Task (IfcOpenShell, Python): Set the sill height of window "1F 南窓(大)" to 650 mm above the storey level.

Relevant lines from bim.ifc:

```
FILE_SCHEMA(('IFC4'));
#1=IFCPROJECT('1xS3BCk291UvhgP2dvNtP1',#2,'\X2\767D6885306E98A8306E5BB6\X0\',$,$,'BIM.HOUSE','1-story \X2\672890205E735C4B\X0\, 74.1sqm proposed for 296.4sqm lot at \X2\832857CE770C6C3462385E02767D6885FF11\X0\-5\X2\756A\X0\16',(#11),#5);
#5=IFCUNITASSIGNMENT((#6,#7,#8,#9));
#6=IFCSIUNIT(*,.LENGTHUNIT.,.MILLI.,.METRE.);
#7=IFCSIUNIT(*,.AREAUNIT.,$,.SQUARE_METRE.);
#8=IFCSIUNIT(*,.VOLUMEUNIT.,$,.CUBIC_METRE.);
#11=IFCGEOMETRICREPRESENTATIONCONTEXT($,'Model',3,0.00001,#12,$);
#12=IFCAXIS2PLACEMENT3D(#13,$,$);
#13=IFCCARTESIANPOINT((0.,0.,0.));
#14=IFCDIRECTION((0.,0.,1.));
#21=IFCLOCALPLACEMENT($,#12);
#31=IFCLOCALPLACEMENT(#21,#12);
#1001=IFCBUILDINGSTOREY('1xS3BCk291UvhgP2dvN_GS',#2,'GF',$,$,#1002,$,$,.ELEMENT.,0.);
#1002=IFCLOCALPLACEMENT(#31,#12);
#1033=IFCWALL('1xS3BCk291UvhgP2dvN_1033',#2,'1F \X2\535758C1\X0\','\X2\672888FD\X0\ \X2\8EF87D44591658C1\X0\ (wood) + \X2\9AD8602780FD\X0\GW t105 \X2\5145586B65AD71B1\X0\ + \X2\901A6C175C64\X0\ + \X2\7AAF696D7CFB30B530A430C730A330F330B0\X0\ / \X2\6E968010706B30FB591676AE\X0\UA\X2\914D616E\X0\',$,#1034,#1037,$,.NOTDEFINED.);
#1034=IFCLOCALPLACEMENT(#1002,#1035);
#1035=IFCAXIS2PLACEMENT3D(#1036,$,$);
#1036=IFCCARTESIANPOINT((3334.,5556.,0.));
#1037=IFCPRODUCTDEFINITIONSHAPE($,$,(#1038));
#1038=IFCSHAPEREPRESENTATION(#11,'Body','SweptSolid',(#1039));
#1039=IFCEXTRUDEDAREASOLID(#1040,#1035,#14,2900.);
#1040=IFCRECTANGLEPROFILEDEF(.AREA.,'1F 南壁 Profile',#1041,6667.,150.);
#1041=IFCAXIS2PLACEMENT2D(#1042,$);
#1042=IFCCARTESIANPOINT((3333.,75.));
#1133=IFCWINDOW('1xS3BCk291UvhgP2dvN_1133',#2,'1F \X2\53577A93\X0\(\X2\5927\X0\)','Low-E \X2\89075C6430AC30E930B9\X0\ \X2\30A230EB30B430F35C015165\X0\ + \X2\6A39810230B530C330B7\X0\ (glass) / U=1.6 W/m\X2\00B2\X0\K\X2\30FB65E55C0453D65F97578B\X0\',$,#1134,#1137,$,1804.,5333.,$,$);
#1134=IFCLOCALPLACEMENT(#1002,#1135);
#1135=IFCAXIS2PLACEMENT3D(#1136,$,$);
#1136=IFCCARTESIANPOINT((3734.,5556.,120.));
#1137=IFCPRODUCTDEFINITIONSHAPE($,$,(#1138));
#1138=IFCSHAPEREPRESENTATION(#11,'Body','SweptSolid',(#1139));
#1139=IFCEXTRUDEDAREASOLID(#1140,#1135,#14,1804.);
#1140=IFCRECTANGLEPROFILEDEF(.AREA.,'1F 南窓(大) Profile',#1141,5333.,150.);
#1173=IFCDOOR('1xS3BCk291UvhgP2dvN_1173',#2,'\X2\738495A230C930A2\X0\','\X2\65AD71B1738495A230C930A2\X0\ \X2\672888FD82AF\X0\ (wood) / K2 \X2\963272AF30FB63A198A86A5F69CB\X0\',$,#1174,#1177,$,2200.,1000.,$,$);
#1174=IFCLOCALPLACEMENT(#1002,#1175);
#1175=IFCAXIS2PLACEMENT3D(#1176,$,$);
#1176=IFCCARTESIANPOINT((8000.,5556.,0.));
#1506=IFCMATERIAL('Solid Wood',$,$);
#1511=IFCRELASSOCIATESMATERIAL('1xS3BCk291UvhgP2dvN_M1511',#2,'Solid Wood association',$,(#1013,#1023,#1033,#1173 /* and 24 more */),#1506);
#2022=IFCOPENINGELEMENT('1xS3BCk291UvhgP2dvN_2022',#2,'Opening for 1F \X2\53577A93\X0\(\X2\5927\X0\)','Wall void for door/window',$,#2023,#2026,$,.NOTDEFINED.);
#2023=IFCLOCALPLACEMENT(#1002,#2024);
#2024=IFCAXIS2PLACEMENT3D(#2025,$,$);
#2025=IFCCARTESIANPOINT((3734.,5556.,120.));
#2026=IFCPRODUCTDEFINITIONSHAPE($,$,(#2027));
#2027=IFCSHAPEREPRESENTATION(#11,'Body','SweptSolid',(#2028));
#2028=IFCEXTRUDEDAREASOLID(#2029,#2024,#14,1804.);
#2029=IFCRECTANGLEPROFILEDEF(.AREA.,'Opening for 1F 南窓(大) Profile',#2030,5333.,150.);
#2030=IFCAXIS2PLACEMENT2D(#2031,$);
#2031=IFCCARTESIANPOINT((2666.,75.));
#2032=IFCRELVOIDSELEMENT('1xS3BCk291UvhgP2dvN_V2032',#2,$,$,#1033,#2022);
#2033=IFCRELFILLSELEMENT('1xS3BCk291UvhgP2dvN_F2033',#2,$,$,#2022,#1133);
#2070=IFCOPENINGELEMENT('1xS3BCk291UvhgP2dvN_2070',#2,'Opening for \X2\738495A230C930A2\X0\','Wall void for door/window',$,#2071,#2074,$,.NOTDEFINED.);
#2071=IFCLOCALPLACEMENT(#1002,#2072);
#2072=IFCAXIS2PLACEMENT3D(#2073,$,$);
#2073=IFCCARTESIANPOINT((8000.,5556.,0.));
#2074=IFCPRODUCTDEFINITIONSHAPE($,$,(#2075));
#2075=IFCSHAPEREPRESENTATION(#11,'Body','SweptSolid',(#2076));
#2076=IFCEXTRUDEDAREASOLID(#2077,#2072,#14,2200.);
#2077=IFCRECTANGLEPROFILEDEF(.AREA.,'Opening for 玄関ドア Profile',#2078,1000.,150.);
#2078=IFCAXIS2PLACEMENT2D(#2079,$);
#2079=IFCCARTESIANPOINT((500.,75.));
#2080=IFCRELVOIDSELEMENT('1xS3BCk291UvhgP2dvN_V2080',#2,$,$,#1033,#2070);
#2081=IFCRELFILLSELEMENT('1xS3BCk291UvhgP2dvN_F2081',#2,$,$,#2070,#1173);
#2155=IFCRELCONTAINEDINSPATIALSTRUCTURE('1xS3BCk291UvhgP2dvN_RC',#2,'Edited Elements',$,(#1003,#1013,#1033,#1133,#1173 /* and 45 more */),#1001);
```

```python
import numpy as np
import ifcopenshell
import ifcopenshell.api.geometry
import ifcopenshell.geom
import ifcopenshell.util.element
import ifcopenshell.util.placement
import ifcopenshell.util.shape
import ifcopenshell.util.unit

model = ifcopenshell.open("bim.ifc")
unit_scale = ifcopenshell.util.unit.calculate_unit_scale(model)

window = model.by_guid("1xS3BCk291UvhgP2dvN_1133")
opening = window.FillsVoids[0].RelatingOpeningElement
storey = ifcopenshell.util.element.get_container(window, ifc_class="IfcBuildingStorey")
level = ifcopenshell.util.placement.get_local_placement(storey.ObjectPlacement)[2, 3]

# The opening's origin need not be at the sill, so measure its lowest point.
shape = ifcopenshell.geom.create_shape(ifcopenshell.geom.settings(), opening)
bottom = ifcopenshell.util.shape.get_shape_bottom_elevation(shape, shape.geometry) / unit_scale
dz = level + 0.65 / unit_scale - bottom

shift = np.array([0.0, 0.0, dz])
# The window is not placed relative to its opening, so move both.
for product in (opening, window):
    matrix = ifcopenshell.util.placement.get_local_placement(product.ObjectPlacement)
    matrix[:3, 3] += shift
    ifcopenshell.api.geometry.edit_object_placement(model, product=product, matrix=matrix, is_si=False)

print(f"moved by {dz * unit_scale:+.3f} m")

model.write("bim_updated.ifc")
```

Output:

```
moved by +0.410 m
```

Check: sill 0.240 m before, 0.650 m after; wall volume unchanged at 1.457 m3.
